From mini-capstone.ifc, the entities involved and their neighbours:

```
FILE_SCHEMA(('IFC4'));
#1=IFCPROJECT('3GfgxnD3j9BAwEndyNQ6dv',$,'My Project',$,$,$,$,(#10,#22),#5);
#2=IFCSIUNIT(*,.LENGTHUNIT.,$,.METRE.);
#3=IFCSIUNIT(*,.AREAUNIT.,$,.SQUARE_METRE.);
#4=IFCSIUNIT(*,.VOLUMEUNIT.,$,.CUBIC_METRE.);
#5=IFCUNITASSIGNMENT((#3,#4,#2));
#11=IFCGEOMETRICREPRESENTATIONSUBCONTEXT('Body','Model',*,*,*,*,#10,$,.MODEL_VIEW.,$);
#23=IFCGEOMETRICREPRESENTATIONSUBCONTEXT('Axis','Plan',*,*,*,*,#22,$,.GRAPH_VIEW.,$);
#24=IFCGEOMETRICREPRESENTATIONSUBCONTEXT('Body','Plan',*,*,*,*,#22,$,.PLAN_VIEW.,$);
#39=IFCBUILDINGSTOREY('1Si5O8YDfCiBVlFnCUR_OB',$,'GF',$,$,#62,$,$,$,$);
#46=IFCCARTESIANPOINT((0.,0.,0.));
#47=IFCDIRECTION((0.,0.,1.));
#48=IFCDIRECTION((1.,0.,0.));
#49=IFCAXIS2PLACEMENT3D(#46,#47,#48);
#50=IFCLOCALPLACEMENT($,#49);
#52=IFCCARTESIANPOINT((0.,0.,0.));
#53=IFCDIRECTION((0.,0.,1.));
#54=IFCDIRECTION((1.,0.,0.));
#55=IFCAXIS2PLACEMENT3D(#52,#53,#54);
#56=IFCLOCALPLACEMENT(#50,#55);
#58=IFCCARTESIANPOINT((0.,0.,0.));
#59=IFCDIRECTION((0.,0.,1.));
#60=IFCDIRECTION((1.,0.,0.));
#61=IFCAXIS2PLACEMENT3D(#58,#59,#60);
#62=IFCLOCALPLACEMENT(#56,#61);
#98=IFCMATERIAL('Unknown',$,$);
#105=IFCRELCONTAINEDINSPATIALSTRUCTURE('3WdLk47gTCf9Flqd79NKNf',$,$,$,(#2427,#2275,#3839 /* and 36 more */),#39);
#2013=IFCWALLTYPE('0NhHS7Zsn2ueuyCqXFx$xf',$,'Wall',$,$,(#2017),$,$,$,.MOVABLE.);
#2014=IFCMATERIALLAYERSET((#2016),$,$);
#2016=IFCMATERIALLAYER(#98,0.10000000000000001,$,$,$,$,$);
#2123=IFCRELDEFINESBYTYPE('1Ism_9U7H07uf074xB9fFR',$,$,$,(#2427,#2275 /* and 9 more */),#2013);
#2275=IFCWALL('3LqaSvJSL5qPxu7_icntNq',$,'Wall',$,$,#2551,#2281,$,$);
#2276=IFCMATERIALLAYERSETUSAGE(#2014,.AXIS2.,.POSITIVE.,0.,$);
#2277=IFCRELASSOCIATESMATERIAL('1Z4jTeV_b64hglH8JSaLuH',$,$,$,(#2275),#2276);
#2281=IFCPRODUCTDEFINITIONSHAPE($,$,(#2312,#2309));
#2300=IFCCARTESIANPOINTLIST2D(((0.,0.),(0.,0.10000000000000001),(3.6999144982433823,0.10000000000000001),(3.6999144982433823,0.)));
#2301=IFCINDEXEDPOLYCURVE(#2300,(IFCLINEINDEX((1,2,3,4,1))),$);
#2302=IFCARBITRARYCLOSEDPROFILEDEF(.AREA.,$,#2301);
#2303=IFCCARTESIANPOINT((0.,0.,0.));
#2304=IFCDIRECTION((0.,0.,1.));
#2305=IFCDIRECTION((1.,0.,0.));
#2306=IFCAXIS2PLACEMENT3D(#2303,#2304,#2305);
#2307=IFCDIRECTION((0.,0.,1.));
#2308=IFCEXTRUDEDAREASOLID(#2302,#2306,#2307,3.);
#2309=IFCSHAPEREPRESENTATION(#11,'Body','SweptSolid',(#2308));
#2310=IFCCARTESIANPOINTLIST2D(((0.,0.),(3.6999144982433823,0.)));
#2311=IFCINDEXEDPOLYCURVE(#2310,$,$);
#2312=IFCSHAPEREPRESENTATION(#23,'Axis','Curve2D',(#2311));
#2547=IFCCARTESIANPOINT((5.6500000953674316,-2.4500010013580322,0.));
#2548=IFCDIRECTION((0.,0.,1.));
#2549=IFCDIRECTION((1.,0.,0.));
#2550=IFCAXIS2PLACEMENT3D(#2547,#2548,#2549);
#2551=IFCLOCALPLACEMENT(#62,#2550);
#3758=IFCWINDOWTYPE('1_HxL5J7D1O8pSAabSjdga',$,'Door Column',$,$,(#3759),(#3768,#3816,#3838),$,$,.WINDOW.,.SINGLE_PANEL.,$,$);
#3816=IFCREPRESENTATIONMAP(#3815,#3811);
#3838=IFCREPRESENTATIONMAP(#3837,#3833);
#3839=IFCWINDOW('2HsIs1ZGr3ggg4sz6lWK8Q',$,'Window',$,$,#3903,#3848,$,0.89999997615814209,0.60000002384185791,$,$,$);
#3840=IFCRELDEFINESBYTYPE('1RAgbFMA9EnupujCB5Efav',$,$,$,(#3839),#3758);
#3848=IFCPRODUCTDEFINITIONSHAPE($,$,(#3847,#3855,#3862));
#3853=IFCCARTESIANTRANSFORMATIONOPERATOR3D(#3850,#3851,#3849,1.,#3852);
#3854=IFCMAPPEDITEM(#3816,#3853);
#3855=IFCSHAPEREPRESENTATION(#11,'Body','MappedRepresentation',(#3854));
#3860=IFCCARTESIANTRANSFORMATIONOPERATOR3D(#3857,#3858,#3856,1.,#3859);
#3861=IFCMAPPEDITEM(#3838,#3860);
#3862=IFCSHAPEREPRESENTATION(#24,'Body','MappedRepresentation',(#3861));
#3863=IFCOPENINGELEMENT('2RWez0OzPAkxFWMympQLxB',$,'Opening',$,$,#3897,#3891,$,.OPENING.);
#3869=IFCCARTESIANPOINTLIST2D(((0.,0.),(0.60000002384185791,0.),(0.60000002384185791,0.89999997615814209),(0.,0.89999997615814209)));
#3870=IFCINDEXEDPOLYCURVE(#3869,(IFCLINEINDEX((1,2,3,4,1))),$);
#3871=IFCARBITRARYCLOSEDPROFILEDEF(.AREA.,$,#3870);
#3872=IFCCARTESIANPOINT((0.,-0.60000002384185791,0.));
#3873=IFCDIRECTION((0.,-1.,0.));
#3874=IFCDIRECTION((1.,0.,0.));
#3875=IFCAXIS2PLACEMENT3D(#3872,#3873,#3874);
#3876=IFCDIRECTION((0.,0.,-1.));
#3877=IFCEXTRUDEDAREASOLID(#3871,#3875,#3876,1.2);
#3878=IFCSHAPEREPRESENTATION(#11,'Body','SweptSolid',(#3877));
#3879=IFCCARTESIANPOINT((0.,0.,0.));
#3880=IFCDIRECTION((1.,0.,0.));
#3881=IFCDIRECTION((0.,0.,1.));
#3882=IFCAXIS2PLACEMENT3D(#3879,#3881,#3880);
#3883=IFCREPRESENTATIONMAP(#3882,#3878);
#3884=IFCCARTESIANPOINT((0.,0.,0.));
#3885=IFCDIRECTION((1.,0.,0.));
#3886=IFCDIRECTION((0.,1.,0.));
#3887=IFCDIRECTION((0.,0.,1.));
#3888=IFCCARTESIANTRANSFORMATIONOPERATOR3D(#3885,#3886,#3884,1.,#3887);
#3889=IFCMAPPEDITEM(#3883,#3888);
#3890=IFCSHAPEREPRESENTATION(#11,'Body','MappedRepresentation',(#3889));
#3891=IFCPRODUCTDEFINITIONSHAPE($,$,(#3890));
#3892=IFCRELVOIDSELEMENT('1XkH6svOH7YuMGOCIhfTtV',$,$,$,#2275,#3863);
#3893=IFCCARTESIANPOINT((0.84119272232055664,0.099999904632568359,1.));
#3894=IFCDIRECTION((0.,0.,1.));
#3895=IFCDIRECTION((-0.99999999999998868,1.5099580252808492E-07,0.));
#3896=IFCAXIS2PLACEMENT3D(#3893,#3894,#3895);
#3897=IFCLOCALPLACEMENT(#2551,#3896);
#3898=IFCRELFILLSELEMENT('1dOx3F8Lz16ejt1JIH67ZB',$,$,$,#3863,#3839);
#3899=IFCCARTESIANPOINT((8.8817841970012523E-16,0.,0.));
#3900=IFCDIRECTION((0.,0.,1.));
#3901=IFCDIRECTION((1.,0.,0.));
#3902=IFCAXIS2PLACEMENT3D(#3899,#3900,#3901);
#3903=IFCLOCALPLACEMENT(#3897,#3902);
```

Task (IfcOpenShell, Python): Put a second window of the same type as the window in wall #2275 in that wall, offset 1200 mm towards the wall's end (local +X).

```python
import ifcopenshell
import ifcopenshell.api.feature
import ifcopenshell.api.geometry
import ifcopenshell.api.root
import ifcopenshell.geom
import ifcopenshell.util.element
import ifcopenshell.util.placement
import ifcopenshell.util.shape
import ifcopenshell.util.unit

model = ifcopenshell.open("mini-capstone.ifc")
unit_scale = ifcopenshell.util.unit.calculate_unit_scale(model)
settings = ifcopenshell.geom.settings()


def volume(element):
    """Net volume in cubic metres, openings subtracted."""
    shape = ifcopenshell.geom.create_shape(settings, element)
    return ifcopenshell.util.shape.get_volume(shape.geometry)


window = model.by_guid("2HsIs1ZGr3ggg4sz6lWK8Q")
opening = window.FillsVoids[0].RelatingOpeningElement
wall = opening.VoidsElements[0].RelatingBuildingElement
before = volume(wall)
shift = ifcopenshell.util.placement.get_local_placement(wall.ObjectPlacement)[:3, 0] * 1.2 / unit_scale

# copy_class copies the void relationship, type, container and properties, but no geometry.
new_opening = ifcopenshell.api.root.copy_class(model, product=opening)
new_opening.Representation = ifcopenshell.util.element.copy_deep(
    model, opening.Representation, exclude=["IfcGeometricRepresentationContext", "IfcRepresentationMap"]
)
new_window = ifcopenshell.api.root.copy_class(model, product=window)
new_window.Representation = ifcopenshell.util.element.copy_deep(
    model, window.Representation, exclude=["IfcGeometricRepresentationContext", "IfcRepresentationMap"]
)
ifcopenshell.api.feature.add_filling(model, opening=new_opening, element=new_window)

for old, new in ((opening, new_opening), (window, new_window)):
    matrix = ifcopenshell.util.placement.get_local_placement(old.ObjectPlacement)
    matrix[:3, 3] += shift
    ifcopenshell.api.geometry.edit_object_placement(model, product=new, matrix=matrix, is_si=False)

after = volume(wall)

print(f"wall volume {before:.3f} -> {after:.3f} m3")

model.write("mini-capstone_rev.ifc")
```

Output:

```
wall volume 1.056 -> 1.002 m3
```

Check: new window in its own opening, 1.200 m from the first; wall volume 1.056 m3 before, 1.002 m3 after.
